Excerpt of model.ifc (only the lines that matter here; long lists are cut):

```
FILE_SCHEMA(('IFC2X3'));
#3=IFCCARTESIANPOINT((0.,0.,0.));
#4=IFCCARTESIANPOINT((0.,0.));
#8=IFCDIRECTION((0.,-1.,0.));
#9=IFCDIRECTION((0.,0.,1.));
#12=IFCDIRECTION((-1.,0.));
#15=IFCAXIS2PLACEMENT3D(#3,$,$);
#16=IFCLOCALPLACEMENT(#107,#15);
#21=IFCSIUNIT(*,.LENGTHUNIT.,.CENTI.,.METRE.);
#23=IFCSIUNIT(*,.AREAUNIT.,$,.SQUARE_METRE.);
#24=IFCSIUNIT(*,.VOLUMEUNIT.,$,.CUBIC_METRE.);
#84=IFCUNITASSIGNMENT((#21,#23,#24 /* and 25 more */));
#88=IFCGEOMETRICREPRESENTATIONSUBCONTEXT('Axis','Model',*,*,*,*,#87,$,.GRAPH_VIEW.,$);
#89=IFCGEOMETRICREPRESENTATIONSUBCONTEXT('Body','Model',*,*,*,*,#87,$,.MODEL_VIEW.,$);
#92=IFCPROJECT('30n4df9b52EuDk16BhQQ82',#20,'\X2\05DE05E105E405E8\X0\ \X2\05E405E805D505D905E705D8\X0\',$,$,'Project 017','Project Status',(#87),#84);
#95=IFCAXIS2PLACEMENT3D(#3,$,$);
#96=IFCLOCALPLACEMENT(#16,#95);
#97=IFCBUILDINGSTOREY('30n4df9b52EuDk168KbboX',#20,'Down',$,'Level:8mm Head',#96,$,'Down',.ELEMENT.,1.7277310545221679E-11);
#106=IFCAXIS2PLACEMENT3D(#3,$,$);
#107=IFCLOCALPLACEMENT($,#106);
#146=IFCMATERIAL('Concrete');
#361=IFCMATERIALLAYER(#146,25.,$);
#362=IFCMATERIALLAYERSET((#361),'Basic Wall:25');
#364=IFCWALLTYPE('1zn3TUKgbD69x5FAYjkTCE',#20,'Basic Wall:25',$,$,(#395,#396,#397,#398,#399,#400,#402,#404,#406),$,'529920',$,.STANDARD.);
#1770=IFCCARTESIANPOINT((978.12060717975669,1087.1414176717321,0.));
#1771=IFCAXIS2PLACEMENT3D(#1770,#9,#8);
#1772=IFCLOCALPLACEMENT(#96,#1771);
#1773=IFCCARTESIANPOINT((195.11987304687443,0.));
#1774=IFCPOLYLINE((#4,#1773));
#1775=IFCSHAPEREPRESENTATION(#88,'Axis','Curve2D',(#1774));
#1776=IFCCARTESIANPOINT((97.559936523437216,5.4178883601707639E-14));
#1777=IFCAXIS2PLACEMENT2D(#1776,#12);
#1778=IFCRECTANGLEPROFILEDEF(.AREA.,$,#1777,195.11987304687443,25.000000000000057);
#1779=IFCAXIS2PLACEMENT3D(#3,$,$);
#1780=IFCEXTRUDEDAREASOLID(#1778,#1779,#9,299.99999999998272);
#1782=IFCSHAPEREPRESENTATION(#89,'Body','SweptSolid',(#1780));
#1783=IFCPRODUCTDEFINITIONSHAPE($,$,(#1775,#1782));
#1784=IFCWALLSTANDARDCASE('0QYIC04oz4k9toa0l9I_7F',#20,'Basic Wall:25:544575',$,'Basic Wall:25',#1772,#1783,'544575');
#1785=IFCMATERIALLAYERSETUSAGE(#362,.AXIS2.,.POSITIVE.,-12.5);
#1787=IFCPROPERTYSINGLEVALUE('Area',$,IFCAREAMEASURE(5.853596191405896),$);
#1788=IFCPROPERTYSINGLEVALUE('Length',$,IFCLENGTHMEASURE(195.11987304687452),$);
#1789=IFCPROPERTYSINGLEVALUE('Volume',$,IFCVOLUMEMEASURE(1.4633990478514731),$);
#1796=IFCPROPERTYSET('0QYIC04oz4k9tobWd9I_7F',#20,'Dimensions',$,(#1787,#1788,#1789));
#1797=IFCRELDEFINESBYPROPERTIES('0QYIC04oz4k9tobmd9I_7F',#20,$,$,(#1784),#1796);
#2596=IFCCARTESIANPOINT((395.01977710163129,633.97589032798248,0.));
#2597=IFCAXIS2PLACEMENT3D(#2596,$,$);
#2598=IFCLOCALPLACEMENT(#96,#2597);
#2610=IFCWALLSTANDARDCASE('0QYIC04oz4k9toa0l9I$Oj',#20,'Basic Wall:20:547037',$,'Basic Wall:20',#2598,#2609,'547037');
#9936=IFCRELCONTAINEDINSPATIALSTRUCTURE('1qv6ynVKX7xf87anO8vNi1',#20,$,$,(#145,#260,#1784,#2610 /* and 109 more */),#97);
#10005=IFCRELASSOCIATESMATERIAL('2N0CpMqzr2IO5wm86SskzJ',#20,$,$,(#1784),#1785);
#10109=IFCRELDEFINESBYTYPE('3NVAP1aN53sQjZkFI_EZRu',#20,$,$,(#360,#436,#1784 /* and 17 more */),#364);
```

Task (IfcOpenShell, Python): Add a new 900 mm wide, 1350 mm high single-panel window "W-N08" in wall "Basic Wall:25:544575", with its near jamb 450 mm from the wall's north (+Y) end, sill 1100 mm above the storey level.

```python
import numpy as np
import ifcopenshell
import ifcopenshell.api.feature
import ifcopenshell.api.geometry
import ifcopenshell.api.pset
import ifcopenshell.api.root
import ifcopenshell.api.spatial
import ifcopenshell.api.type
import ifcopenshell.geom
import ifcopenshell.util.element
import ifcopenshell.util.placement
import ifcopenshell.util.representation
import ifcopenshell.util.shape
import ifcopenshell.util.unit

model = ifcopenshell.open("model.ifc")
unit_scale = ifcopenshell.util.unit.calculate_unit_scale(model)
area_scale = ifcopenshell.util.unit.calculate_unit_scale(model, "AREAUNIT")
volume_scale = ifcopenshell.util.unit.calculate_unit_scale(model, "VOLUMEUNIT")
settings = ifcopenshell.geom.settings()


def volume(element):
    """Net volume in cubic metres, openings subtracted."""
    shape = ifcopenshell.geom.create_shape(settings, element)
    return ifcopenshell.util.shape.get_volume(shape.geometry)


wall = model.by_guid("0QYIC04oz4k9toa0l9I_7F")
storey = ifcopenshell.util.element.get_container(wall, ifc_class="IfcBuildingStorey")
context = ifcopenshell.util.representation.get_context(model, "Model", "Body", "MODEL_VIEW")
before = volume(wall)

width, height, from_end, sill = 0.9, 1.35, 0.45, 1.1  # metres

# The wall runs along its own X axis, and the end named is its -X end.
wall_shape = ifcopenshell.geom.create_shape(settings, wall)
x, y, z = ifcopenshell.util.shape.get_vertices(wall_shape.geometry).T
start = x.min() + from_end
face, thickness = float(y.min()), float(y.max() - y.min())
wall_matrix = ifcopenshell.util.placement.get_local_placement(wall.ObjectPlacement)
level = ifcopenshell.util.placement.get_local_placement(storey.ObjectPlacement)[2, 3]


def in_wall(x, y):
    """Placement at x, y metres in the wall's axes, at sill height."""
    matrix = wall_matrix.copy()
    matrix[:, 3] = wall_matrix @ np.array([x / unit_scale, y / unit_scale, 0.0, 1.0])
    matrix[2, 3] = level + sill / unit_scale
    return matrix


# Opening: a box that overshoots both wall faces by 50 mm.
opening = ifcopenshell.api.root.create_entity(model, ifc_class="IfcOpeningElement")
box = ifcopenshell.api.geometry.add_wall_representation(
    model, context=context, length=width, height=height, thickness=thickness + 0.1
)
ifcopenshell.api.geometry.assign_representation(model, product=opening, representation=box)
ifcopenshell.api.geometry.edit_object_placement(model, product=opening, matrix=in_wall(start, face - 0.05), is_si=False)
ifcopenshell.api.feature.add_feature(model, feature=opening, element=wall)

window = ifcopenshell.api.root.create_entity(model, ifc_class="IfcWindow", name="W-N08")
window.OverallWidth, window.OverallHeight = width / unit_scale, height / unit_scale
body = ifcopenshell.api.geometry.add_window_representation(
    model,
    context=context,
    overall_width=window.OverallWidth,
    overall_height=window.OverallHeight,
    partition_type="SINGLE_PANEL",
)
ifcopenshell.api.geometry.assign_representation(model, product=window, representation=body)
ifcopenshell.api.spatial.assign_container(model, products=[window], relating_structure=storey)
fills = ifcopenshell.api.feature.add_filling(model, opening=opening, element=window)
fills.OwnerHistory = window.OwnerHistory  # required in IFC2X3

# IFC2X3 keeps the operation on the window style.
style = ifcopenshell.api.root.create_entity(model, ifc_class="IfcWindowStyle", name="W-N08")
style.OperationType, style.ConstructionType = "SINGLE_PANEL", "NOTDEFINED"
style.ParameterTakesPrecedence = style.Sizeable = False
ifcopenshell.api.type.assign_type(model, related_objects=[window], relating_type=style)

# Centre the window in the wall's thickness.
ifcopenshell.api.geometry.edit_object_placement(model, product=window, matrix=in_wall(start, face), is_si=False)
window_shape = ifcopenshell.geom.create_shape(settings, window)
depth = ifcopenshell.util.shape.get_vertices(window_shape.geometry)[:, 1]
offset = face + thickness / 2 - (depth.min() + depth.max()) / 2
ifcopenshell.api.geometry.edit_object_placement(model, product=window, matrix=in_wall(start, offset), is_si=False)

after = volume(wall)

# Update the wall's stored quantities.
pset = model.by_id(ifcopenshell.util.element.get_pset(wall, "Dimensions", should_inherit=False)["id"])
ifcopenshell.api.pset.edit_pset(model, pset=pset, properties={
    "Area": model.create_entity("IfcAreaMeasure", after / thickness / area_scale),
    "Volume": model.create_entity("IfcVolumeMeasure", after / volume_scale),
})

print(f"wall volume {before:.3f} -> {after:.3f} m3")

model.write("model_edited.ifc")
```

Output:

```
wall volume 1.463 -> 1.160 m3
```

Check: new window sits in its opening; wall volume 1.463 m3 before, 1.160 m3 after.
